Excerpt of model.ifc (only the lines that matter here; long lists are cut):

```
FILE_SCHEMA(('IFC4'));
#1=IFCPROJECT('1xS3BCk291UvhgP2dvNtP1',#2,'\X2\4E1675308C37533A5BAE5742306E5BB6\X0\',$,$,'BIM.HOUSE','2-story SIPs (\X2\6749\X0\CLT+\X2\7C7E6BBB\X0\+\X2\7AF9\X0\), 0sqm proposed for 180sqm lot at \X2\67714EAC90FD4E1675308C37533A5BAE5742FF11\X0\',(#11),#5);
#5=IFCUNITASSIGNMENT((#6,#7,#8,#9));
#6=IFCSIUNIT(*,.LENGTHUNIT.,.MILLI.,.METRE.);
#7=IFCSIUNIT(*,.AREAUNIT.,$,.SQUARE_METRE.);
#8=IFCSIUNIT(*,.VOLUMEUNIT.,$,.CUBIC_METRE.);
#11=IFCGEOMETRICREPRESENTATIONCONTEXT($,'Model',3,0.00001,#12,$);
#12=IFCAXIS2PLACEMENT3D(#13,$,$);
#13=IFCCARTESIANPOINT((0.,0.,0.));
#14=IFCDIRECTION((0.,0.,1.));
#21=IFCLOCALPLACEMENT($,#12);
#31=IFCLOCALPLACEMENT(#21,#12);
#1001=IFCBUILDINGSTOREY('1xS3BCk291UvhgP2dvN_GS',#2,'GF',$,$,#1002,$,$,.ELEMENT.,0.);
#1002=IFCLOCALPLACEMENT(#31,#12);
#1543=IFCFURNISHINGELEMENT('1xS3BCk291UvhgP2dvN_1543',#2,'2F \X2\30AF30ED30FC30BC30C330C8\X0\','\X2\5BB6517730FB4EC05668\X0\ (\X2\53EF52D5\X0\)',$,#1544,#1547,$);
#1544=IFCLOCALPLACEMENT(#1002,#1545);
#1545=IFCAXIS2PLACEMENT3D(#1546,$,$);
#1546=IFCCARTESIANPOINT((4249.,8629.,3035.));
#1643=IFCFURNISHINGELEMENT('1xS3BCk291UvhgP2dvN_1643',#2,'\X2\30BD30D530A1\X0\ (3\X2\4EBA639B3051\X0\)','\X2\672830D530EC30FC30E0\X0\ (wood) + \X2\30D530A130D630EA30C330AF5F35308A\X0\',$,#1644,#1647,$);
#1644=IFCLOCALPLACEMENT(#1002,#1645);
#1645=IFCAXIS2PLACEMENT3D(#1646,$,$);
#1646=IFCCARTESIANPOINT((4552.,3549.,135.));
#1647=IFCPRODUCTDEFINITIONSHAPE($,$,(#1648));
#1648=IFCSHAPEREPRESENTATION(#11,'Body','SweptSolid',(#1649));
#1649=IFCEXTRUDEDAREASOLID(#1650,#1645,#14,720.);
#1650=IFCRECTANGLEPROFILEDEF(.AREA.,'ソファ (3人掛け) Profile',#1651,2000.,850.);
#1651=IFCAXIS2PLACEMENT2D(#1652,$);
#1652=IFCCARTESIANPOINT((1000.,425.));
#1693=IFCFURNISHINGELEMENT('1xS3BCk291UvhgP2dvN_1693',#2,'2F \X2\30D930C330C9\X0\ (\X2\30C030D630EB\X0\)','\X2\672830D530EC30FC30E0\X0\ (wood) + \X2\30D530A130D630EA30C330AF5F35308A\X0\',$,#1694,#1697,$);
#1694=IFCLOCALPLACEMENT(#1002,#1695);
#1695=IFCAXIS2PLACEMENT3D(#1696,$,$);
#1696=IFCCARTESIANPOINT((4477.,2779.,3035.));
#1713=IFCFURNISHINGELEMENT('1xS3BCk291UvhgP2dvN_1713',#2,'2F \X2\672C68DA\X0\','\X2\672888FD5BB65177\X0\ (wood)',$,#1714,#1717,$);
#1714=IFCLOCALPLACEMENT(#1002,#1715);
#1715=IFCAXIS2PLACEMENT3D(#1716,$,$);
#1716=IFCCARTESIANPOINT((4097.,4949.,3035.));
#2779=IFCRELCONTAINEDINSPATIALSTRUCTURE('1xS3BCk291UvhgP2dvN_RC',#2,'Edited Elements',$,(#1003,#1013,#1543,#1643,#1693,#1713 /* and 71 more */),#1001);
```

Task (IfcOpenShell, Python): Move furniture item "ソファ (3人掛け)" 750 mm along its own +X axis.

```python
import ifcopenshell
import ifcopenshell.api.geometry
import ifcopenshell.util.placement

model = ifcopenshell.open("model.ifc")

item = model.by_guid("1xS3BCk291UvhgP2dvN_1643")
matrix = ifcopenshell.util.placement.get_local_placement(item.ObjectPlacement)
matrix[:3, 3] += matrix[:3, 0] * 750.0
ifcopenshell.api.geometry.edit_object_placement(model, product=item, matrix=matrix, is_si=False)

print(ifcopenshell.util.placement.get_local_placement(item.ObjectPlacement).round(3) + 0.0)

model.write("model-out.ifc")
```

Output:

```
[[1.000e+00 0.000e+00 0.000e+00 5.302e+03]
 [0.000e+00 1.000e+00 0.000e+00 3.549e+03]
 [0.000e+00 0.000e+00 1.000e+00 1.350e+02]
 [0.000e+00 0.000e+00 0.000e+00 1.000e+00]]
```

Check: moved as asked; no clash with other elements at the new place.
